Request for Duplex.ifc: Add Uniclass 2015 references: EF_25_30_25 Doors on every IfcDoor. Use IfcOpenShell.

First a look at what the model holds.

```python
import ifcopenshell

model = ifcopenshell.open("Duplex.ifc")
print(model.schema)
print("classifications:", [c.Name for c in model.by_type("IfcClassification")])
for ifc_class in ("IfcDoor", "IfcRoof", "IfcStair", "IfcWall", "IfcWindow"):
    print(ifc_class, len(model.by_type(ifc_class)))
```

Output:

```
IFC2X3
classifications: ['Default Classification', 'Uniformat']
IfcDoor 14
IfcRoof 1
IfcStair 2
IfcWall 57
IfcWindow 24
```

```python
import ifcopenshell
import ifcopenshell.api.classification

model = ifcopenshell.open("Duplex.ifc")

# IFC2X3 requires Source and Edition and has no link from the project to the system.
system = model.create_entity("IfcClassification", Source="NBS", Edition="2015", Name="Uniclass 2015")

codes = {
    "IfcDoor": ("EF_25_30_25", "Doors"),
}
for ifc_class, (code, name) in codes.items():
    products = model.by_type(ifc_class)
    ifcopenshell.api.classification.add_reference(
        model, products=products, classification=system, identification=code, name=name
    )
    print(code, len(products))

model.write("Duplex_rev.ifc")
```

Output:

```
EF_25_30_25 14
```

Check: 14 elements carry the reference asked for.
